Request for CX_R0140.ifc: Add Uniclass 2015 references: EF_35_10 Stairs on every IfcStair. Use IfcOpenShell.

First a look at what the model holds.

```python
import ifcopenshell

model = ifcopenshell.open("CX_R0140.ifc")
print(model.schema)
print("classifications:", [c.Name for c in model.by_type("IfcClassification")])
for ifc_class in ("IfcDoor", "IfcRoof", "IfcStair", "IfcWall", "IfcWindow"):
    print(ifc_class, len(model.by_type(ifc_class)))
```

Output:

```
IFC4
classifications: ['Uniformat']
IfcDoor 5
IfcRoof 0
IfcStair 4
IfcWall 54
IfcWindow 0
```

```python
import ifcopenshell
import ifcopenshell.api.classification

model = ifcopenshell.open("CX_R0140.ifc")

system = ifcopenshell.api.classification.add_classification(model, classification="Uniclass 2015")

codes = {
    "IfcStair": ("EF_35_10", "Stairs"),
}
for ifc_class, (code, name) in codes.items():
    products = model.by_type(ifc_class)
    ifcopenshell.api.classification.add_reference(
        model, products=products, classification=system, identification=code, name=name
    )
    print(code, len(products))

model.write("CX_R0140-out.ifc")
```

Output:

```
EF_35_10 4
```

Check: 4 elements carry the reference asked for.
